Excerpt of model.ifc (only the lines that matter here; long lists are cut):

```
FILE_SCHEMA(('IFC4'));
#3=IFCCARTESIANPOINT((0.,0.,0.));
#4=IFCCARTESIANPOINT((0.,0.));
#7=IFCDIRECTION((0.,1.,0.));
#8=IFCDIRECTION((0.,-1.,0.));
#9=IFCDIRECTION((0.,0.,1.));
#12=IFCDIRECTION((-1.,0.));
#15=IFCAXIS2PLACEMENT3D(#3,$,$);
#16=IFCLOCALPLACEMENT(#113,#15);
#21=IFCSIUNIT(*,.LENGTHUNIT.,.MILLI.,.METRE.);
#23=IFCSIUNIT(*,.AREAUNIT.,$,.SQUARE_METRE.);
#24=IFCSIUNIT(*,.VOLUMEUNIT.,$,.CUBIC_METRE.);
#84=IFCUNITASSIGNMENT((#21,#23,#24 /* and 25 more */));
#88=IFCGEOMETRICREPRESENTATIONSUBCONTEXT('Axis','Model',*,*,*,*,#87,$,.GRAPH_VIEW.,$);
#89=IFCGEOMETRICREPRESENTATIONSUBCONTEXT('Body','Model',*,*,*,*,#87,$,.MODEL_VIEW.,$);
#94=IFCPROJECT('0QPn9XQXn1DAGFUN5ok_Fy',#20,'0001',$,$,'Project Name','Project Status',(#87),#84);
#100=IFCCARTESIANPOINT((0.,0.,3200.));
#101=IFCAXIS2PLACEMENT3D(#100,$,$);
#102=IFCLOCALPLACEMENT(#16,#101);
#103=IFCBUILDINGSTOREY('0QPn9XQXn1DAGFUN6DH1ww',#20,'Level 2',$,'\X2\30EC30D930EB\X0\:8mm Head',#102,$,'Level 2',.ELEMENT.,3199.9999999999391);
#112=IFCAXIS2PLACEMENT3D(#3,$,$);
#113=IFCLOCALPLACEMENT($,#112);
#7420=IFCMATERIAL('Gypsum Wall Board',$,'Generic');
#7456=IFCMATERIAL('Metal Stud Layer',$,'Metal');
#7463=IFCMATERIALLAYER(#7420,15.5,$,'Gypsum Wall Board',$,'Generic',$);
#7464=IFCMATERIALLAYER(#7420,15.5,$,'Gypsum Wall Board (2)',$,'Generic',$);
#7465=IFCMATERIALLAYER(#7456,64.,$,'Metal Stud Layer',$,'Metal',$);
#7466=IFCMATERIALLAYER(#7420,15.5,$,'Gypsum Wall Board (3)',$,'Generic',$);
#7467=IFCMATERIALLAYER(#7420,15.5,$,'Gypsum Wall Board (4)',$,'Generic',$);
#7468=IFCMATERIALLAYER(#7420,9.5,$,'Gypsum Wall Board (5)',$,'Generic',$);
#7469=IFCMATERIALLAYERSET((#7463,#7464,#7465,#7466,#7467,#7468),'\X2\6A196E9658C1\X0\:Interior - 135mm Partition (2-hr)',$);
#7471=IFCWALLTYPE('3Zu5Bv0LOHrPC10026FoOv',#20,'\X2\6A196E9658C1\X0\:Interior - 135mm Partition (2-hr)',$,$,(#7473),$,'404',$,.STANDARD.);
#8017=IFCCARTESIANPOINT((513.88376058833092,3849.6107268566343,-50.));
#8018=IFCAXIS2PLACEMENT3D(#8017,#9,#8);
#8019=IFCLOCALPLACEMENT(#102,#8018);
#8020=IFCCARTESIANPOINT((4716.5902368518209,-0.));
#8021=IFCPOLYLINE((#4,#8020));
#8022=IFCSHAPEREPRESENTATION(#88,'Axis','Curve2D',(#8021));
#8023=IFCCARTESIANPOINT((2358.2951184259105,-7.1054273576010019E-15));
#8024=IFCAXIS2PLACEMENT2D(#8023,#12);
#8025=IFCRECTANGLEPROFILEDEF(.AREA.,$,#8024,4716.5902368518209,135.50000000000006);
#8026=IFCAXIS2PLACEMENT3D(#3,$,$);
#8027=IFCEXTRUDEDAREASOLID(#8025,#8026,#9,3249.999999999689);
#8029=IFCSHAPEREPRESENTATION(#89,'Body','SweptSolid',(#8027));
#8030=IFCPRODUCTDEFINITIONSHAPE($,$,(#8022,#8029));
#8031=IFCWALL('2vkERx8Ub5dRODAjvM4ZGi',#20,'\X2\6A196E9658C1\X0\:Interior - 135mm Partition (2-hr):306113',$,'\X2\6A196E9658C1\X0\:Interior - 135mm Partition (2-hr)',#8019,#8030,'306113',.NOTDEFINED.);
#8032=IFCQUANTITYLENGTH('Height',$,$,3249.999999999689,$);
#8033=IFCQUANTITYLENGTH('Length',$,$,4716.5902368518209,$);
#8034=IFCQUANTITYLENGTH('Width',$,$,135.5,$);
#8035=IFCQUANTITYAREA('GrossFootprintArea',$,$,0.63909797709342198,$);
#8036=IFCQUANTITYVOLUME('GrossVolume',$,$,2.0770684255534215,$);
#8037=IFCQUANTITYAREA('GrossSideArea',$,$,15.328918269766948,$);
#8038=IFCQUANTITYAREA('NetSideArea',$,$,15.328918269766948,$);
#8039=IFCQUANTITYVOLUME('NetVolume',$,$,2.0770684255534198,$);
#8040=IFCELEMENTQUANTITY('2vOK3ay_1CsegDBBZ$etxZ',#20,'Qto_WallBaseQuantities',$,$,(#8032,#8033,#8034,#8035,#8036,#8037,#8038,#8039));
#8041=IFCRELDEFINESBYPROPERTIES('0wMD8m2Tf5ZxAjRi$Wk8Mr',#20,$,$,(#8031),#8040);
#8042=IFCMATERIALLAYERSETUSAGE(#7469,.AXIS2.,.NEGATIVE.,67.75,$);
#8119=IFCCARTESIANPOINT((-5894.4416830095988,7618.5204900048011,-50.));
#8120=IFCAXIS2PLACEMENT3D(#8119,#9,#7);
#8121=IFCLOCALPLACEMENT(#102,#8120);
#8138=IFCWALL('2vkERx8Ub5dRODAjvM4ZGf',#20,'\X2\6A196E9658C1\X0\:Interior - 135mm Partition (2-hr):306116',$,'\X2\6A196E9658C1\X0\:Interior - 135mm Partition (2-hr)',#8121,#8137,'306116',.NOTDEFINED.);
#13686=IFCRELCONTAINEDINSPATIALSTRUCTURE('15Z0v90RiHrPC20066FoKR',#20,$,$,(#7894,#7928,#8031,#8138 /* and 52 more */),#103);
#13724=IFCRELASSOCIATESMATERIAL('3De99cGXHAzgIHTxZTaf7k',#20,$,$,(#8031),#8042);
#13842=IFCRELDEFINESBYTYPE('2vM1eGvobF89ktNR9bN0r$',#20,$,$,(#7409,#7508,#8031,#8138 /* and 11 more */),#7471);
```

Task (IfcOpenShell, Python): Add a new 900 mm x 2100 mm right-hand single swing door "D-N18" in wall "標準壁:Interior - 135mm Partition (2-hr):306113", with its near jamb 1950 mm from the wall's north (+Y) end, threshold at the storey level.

```python
import numpy as np
import ifcopenshell
import ifcopenshell.api.feature
import ifcopenshell.api.geometry
import ifcopenshell.api.pset
import ifcopenshell.api.root
import ifcopenshell.api.spatial
import ifcopenshell.geom
import ifcopenshell.util.element
import ifcopenshell.util.placement
import ifcopenshell.util.representation
import ifcopenshell.util.shape
import ifcopenshell.util.unit

model = ifcopenshell.open("model.ifc")
unit_scale = ifcopenshell.util.unit.calculate_unit_scale(model)
area_scale = ifcopenshell.util.unit.calculate_unit_scale(model, "AREAUNIT")
volume_scale = ifcopenshell.util.unit.calculate_unit_scale(model, "VOLUMEUNIT")
settings = ifcopenshell.geom.settings()


def volume(element):
    """Net volume in cubic metres, openings subtracted."""
    shape = ifcopenshell.geom.create_shape(settings, element)
    return ifcopenshell.util.shape.get_volume(shape.geometry)


wall = model.by_guid("2vkERx8Ub5dRODAjvM4ZGi")
storey = ifcopenshell.util.element.get_container(wall, ifc_class="IfcBuildingStorey")
context = ifcopenshell.util.representation.get_context(model, "Model", "Body", "MODEL_VIEW")
before = volume(wall)

width, height, from_end, sill = 0.9, 2.1, 1.95, 0.0  # metres

# The wall runs along its own X axis, and the end named is its -X end.
wall_shape = ifcopenshell.geom.create_shape(settings, wall)
x, y, z = ifcopenshell.util.shape.get_vertices(wall_shape.geometry).T
start = x.min() + from_end
face, thickness = float(y.min()), float(y.max() - y.min())
wall_matrix = ifcopenshell.util.placement.get_local_placement(wall.ObjectPlacement)
level = ifcopenshell.util.placement.get_local_placement(storey.ObjectPlacement)[2, 3]


def in_wall(x, y):
    """Placement at x, y metres in the wall's axes, at sill height."""
    matrix = wall_matrix.copy()
    matrix[:, 3] = wall_matrix @ np.array([x / unit_scale, y / unit_scale, 0.0, 1.0])
    matrix[2, 3] = level + sill / unit_scale
    return matrix


# Opening: a box that overshoots both wall faces by 50 mm.
opening = ifcopenshell.api.root.create_entity(model, ifc_class="IfcOpeningElement", predefined_type="OPENING")
box = ifcopenshell.api.geometry.add_wall_representation(
    model, context=context, length=width, height=height, thickness=thickness + 0.1
)
ifcopenshell.api.geometry.assign_representation(model, product=opening, representation=box)
ifcopenshell.api.geometry.edit_object_placement(model, product=opening, matrix=in_wall(start, face - 0.05), is_si=False)
ifcopenshell.api.feature.add_feature(model, feature=opening, element=wall)

door = ifcopenshell.api.root.create_entity(model, ifc_class="IfcDoor", name="D-N18", predefined_type="DOOR")
door.OverallWidth, door.OverallHeight = width / unit_scale, height / unit_scale
door.OperationType = "SINGLE_SWING_RIGHT"
body = ifcopenshell.api.geometry.add_door_representation(
    model,
    context=context,
    overall_width=door.OverallWidth,
    overall_height=door.OverallHeight,
    operation_type="SINGLE_SWING_RIGHT",
    lining_properties={"LiningDepth": thickness / unit_scale, "ThresholdDepth": thickness / unit_scale},
)
ifcopenshell.api.geometry.assign_representation(model, product=door, representation=body)
ifcopenshell.api.spatial.assign_container(model, products=[door], relating_structure=storey)
ifcopenshell.api.feature.add_filling(model, opening=opening, element=door)

# The lining spans the wall, so the door starts at the wall face.
ifcopenshell.api.geometry.edit_object_placement(model, product=door, matrix=in_wall(start, face), is_si=False)

after = volume(wall)

# Update the wall's stored quantities.
qto = model.by_id(ifcopenshell.util.element.get_pset(wall, "Qto_WallBaseQuantities", should_inherit=False)["id"])
ifcopenshell.api.pset.edit_qto(model, qto=qto, properties={
    "NetSideArea": after / thickness / area_scale,
    "NetVolume": after / volume_scale,
})

print(f"wall volume {before:.3f} -> {after:.3f} m3")

model.write("model_edited.ifc")
```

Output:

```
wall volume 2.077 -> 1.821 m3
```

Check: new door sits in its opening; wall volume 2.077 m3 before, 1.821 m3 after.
